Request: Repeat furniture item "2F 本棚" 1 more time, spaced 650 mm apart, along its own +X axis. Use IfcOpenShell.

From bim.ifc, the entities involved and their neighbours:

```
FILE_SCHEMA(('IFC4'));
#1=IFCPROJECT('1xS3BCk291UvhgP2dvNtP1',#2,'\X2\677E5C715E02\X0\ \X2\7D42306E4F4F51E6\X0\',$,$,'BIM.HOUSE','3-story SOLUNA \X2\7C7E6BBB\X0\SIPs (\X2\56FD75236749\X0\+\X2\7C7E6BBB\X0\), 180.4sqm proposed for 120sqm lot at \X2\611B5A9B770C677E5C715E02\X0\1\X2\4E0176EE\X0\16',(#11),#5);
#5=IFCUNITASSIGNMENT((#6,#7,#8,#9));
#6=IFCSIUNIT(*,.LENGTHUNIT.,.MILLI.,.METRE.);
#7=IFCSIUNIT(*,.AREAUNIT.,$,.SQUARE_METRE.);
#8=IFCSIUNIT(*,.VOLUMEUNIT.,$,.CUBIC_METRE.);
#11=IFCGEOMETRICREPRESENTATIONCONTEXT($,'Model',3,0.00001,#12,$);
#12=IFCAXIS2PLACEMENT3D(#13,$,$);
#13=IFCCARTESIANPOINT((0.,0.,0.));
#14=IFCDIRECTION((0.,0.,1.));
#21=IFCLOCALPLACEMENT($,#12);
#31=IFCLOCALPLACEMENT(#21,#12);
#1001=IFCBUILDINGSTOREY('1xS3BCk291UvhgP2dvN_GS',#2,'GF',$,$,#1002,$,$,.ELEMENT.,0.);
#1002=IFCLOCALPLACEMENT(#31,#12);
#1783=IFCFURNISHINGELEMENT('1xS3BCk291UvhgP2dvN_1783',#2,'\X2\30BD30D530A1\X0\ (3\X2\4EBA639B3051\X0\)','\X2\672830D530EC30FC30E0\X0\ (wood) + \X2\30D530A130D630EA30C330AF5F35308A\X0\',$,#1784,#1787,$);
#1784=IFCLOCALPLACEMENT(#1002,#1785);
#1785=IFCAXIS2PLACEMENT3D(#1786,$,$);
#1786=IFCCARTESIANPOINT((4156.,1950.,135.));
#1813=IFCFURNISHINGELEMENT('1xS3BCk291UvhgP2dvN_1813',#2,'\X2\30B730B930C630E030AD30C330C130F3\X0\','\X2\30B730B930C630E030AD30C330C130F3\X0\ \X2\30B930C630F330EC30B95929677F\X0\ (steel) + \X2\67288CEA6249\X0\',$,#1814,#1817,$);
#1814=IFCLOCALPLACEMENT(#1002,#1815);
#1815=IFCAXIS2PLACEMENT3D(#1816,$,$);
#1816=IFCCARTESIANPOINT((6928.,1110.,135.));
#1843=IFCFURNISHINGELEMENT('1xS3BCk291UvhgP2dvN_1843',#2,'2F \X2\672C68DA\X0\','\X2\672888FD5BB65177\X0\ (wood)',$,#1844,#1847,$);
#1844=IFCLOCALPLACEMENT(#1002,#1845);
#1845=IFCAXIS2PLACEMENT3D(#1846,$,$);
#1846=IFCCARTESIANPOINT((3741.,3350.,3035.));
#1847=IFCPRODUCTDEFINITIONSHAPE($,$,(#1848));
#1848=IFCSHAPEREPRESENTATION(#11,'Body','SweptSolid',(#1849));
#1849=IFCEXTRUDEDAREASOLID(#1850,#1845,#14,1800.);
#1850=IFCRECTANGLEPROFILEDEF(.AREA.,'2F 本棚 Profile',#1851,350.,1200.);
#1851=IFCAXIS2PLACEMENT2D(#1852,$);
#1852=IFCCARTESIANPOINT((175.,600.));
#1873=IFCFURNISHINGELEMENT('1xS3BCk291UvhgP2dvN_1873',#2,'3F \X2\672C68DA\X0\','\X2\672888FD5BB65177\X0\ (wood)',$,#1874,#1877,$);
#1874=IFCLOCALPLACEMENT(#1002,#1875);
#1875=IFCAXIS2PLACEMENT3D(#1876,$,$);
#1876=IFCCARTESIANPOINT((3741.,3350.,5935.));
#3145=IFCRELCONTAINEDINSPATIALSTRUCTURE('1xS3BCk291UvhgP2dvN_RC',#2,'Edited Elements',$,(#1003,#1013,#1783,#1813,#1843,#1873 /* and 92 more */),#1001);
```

```python
import ifcopenshell
import ifcopenshell.api.geometry
import ifcopenshell.api.root
import ifcopenshell.util.element
import ifcopenshell.util.placement

model = ifcopenshell.open("bim.ifc")


def reuse_history(source, copy):
    """copy_class also copies each property set's owner history, people and application; keep the originals."""
    for rel in copy.IsDefinedBy:
        if rel.is_a("IfcRelDefinesByProperties") and (history := rel.RelatingPropertyDefinition.OwnerHistory):
            rel.RelatingPropertyDefinition.OwnerHistory = source.OwnerHistory
            ifcopenshell.util.element.remove_deep2(model, history)


source = model.by_guid("1xS3BCk291UvhgP2dvN_1843")
base = ifcopenshell.util.placement.get_local_placement(source.ObjectPlacement)
step = base[:3, 0] * 650.0

for i in range(1, 2):
    copy = ifcopenshell.api.root.copy_class(model, product=source)
    copy.Representation = ifcopenshell.util.element.copy_deep(
        model, source.Representation, exclude=["IfcGeometricRepresentationContext", "IfcRepresentationMap"]
    )
    reuse_history(source, copy)
    matrix = base.copy()
    matrix[:3, 3] += i * step
    print("added at", matrix[:3, 3].round(3) + 0.0)
    ifcopenshell.api.geometry.edit_object_placement(model, product=copy, matrix=matrix, is_si=False)

model.write("bim-out.ifc")
```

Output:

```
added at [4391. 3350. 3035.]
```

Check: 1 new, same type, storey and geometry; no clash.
